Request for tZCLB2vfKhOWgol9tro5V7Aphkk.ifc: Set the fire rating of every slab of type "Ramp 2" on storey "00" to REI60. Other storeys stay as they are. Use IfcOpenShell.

First a look at what the model holds.

```python
import ifcopenshell
import ifcopenshell.util.element

model = ifcopenshell.open("tZCLB2vfKhOWgol9tro5V7Aphkk.ifc")
print(model.schema)
storey = next(s for s in model.by_type("IfcBuildingStorey") if s.Name == "00")
slabs = [e for e in ifcopenshell.util.element.get_decomposition(storey) if e.is_a("IfcSlab")]
seen = {}
for e in slabs:
    element_type = ifcopenshell.util.element.get_type(e)
    key = (element_type.Name if element_type != e and element_type else None, ifcopenshell.util.element.get_pset(e, "Pset_SlabCommon", "FireRating"))
    seen[key] = seen.get(key, 0) + 1
for (name, value), count in sorted(seen.items(), key=str):
    print(count, "x", name, "|", value)
```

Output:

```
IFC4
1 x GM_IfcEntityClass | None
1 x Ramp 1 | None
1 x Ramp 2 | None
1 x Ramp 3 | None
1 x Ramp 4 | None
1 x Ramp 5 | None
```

```python
import ifcopenshell
import ifcopenshell.api.pset
import ifcopenshell.util.element

model = ifcopenshell.open("tZCLB2vfKhOWgol9tro5V7Aphkk.ifc")

storey = next(s for s in model.by_type("IfcBuildingStorey") if s.Name == "00")
slabs = [e for e in ifcopenshell.util.element.get_decomposition(storey) if e.is_a("IfcSlab")]

count = 0
for e in slabs:
    element_type = ifcopenshell.util.element.get_type(e)
    if element_type in (None, e) or element_type.Name != "Ramp 2":
        continue
    # add_pset returns the element's existing set when there is one.
    pset = ifcopenshell.api.pset.add_pset(model, product=e, name="Pset_SlabCommon")
    ifcopenshell.api.pset.edit_pset(model, pset=pset, properties={"FireRating": "REI60"})
    count += 1

print(count, "slabs updated")

model.write("tZCLB2vfKhOWgol9tro5V7Aphkk_edited.ifc")
```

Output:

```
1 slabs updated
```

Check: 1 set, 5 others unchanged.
